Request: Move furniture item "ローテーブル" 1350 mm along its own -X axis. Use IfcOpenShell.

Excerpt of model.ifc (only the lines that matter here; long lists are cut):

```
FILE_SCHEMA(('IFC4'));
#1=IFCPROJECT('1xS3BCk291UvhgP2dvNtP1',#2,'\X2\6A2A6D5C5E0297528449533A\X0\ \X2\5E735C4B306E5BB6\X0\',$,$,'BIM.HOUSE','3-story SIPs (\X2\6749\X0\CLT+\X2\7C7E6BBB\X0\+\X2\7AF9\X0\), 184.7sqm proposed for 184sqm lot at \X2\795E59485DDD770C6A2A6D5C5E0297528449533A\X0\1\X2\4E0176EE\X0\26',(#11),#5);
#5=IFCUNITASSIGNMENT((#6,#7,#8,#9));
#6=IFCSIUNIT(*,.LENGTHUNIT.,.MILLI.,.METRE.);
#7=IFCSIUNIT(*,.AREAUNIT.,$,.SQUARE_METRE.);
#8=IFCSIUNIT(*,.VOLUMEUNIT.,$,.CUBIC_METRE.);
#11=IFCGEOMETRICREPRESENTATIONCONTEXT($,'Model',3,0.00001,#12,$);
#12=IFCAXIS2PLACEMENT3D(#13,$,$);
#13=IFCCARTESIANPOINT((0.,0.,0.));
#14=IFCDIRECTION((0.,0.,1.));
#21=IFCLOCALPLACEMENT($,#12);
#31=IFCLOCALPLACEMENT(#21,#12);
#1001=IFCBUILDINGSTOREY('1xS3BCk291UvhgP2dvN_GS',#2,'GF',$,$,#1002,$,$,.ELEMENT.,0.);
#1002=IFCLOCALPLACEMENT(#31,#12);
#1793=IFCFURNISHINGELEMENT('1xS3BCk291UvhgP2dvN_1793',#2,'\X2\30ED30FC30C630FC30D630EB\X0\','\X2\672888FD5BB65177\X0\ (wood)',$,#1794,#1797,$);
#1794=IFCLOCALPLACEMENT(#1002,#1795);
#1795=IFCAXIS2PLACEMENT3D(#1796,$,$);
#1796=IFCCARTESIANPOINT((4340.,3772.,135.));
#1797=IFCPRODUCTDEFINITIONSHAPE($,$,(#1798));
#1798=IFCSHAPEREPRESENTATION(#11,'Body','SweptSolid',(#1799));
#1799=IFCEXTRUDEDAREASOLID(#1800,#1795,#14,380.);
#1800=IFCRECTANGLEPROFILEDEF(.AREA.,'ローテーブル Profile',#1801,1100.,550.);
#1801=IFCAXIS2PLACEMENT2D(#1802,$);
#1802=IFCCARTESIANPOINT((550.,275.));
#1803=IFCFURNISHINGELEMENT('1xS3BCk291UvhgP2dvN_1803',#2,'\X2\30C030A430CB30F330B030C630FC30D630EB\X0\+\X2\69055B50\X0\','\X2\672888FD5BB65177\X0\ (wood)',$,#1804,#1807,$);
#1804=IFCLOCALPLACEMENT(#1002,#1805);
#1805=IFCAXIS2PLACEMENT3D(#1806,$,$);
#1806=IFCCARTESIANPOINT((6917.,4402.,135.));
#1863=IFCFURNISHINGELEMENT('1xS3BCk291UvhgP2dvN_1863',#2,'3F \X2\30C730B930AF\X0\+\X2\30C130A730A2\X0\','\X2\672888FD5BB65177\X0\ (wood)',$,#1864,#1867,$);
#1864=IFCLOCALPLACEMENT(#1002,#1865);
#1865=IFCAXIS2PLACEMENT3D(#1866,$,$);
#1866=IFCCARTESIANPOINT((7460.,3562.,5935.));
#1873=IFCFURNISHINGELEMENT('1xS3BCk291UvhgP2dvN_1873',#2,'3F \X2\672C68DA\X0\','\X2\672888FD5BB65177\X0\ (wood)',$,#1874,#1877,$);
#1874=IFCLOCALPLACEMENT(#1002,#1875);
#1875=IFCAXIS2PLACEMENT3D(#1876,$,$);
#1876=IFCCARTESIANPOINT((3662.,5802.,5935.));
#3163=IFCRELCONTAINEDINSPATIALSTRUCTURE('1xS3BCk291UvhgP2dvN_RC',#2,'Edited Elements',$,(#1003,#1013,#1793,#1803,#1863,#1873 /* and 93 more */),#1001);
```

```python
import ifcopenshell
import ifcopenshell.api.geometry
import ifcopenshell.util.placement

model = ifcopenshell.open("model.ifc")

item = model.by_guid("1xS3BCk291UvhgP2dvN_1793")
matrix = ifcopenshell.util.placement.get_local_placement(item.ObjectPlacement)
matrix[:3, 3] -= matrix[:3, 0] * 1350.0
ifcopenshell.api.geometry.edit_object_placement(model, product=item, matrix=matrix, is_si=False)

print(ifcopenshell.util.placement.get_local_placement(item.ObjectPlacement).round(3) + 0.0)

model.write("model_edited.ifc")
```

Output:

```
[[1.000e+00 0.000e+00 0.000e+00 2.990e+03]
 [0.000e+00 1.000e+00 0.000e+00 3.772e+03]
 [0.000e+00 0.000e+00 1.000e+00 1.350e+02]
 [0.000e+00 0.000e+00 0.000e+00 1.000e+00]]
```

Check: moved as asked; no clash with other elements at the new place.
